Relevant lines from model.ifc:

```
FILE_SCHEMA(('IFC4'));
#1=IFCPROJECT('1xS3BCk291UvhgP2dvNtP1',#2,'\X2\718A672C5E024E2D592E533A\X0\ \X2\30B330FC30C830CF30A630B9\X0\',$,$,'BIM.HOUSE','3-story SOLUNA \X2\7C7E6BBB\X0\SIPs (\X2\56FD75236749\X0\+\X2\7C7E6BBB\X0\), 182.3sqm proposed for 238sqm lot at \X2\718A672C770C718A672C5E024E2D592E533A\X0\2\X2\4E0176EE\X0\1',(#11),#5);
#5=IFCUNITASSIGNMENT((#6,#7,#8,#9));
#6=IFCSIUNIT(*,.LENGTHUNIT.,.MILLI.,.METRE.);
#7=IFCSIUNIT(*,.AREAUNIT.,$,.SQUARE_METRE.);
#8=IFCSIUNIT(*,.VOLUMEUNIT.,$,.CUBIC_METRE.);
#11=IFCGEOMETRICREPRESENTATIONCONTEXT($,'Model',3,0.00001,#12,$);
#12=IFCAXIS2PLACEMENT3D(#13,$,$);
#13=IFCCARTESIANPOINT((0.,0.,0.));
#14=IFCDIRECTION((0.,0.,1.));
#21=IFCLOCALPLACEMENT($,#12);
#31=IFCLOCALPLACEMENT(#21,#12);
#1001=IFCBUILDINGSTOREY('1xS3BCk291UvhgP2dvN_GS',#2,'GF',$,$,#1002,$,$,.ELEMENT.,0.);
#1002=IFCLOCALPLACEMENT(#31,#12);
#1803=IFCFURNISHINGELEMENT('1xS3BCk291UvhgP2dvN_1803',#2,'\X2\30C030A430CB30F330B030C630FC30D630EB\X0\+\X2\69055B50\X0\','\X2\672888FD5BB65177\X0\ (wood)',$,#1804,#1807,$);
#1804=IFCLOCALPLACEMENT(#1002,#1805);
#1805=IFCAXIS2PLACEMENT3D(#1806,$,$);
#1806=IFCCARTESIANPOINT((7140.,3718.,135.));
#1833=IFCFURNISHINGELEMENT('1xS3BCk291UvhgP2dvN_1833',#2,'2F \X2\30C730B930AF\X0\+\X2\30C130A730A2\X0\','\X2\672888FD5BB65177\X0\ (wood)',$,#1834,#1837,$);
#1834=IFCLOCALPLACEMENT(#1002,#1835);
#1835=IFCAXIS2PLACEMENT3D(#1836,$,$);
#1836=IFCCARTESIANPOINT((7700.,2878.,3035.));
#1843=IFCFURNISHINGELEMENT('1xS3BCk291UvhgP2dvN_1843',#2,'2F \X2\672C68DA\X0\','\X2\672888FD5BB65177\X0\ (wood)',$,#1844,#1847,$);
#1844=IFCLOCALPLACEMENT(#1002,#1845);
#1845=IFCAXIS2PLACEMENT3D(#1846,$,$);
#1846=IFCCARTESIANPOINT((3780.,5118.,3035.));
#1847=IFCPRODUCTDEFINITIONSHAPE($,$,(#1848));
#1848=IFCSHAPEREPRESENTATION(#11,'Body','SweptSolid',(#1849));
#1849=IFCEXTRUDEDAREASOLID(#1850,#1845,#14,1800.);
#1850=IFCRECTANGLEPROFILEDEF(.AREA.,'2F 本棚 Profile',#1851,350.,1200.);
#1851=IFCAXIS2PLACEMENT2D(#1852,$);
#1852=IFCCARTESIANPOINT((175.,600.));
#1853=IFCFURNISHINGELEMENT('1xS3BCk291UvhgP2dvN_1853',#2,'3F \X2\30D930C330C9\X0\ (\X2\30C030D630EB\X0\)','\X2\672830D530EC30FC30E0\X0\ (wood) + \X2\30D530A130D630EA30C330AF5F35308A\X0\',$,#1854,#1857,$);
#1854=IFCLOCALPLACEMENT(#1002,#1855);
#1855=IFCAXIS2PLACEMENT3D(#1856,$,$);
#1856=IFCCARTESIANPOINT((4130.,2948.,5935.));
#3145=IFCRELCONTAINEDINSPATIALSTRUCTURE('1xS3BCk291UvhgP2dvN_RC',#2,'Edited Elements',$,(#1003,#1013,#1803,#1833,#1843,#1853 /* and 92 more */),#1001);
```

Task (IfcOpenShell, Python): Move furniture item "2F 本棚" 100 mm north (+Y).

```python
import ifcopenshell
import ifcopenshell.api.geometry
import ifcopenshell.util.placement

model = ifcopenshell.open("model.ifc")

item = model.by_guid("1xS3BCk291UvhgP2dvN_1843")
matrix = ifcopenshell.util.placement.get_local_placement(item.ObjectPlacement)
matrix[1, 3] += 100.0
ifcopenshell.api.geometry.edit_object_placement(model, product=item, matrix=matrix, is_si=False)

print(ifcopenshell.util.placement.get_local_placement(item.ObjectPlacement).round(3) + 0.0)

model.write("model_updated.ifc")
```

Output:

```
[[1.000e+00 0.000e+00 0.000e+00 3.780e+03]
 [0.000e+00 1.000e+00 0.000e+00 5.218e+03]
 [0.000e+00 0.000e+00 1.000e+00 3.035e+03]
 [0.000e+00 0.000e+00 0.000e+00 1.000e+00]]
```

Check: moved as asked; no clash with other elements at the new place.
